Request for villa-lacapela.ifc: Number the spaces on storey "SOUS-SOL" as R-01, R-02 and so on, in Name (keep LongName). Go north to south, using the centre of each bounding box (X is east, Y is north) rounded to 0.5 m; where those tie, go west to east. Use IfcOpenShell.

First a look at what the model holds.

```python
import ifcopenshell
import ifcopenshell.util.element
import ifcopenshell.util.placement

model = ifcopenshell.open("villa-lacapela.ifc")
print(model.schema)
storey = next(s for s in model.by_type("IfcBuildingStorey") if s.Name == "SOUS-SOL")
spaces = [e for e in ifcopenshell.util.element.get_decomposition(storey) if e.is_a("IfcSpace")]
for e in sorted(spaces, key=lambda e: e.id()):
    origin = ifcopenshell.util.placement.get_local_placement(e.ObjectPlacement)[:3, 3]
    print(e.id(), e.Name, e.LongName, origin.round(2) + 0.0, sep=" | ")
```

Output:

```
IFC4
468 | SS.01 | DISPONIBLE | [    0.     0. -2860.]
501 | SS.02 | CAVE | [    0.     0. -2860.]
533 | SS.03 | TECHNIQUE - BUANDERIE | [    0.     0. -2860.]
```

```python
import ifcopenshell
import ifcopenshell.geom
import ifcopenshell.util.element
import ifcopenshell.util.shape

model = ifcopenshell.open("villa-lacapela.ifc")
settings = ifcopenshell.geom.settings()
settings.set("use-world-coords", True)


def centre(element):
    shape = ifcopenshell.geom.create_shape(settings, element)
    return ifcopenshell.util.shape.get_bbox_centroid(shape.geometry)


storey = next(s for s in model.by_type("IfcBuildingStorey") if s.Name == "SOUS-SOL")
spaces = [e for e in ifcopenshell.util.element.get_decomposition(storey) if e.is_a("IfcSpace")]

# Insertion points can sit at a corner or the storey origin, so sort by the geometry (in metres).
centres = {e: centre(e) for e in spaces}
spaces.sort(key=lambda e: (-round(centres[e][1] / 0.5), centres[e][0]))

for i, e in enumerate(spaces, start=1):
    number = f"R-{i:02d}"
    e.Name = number
    print(e.id(), number)

model.write("villa-lacapela_edited.ifc")
```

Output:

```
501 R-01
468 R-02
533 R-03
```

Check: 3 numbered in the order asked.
